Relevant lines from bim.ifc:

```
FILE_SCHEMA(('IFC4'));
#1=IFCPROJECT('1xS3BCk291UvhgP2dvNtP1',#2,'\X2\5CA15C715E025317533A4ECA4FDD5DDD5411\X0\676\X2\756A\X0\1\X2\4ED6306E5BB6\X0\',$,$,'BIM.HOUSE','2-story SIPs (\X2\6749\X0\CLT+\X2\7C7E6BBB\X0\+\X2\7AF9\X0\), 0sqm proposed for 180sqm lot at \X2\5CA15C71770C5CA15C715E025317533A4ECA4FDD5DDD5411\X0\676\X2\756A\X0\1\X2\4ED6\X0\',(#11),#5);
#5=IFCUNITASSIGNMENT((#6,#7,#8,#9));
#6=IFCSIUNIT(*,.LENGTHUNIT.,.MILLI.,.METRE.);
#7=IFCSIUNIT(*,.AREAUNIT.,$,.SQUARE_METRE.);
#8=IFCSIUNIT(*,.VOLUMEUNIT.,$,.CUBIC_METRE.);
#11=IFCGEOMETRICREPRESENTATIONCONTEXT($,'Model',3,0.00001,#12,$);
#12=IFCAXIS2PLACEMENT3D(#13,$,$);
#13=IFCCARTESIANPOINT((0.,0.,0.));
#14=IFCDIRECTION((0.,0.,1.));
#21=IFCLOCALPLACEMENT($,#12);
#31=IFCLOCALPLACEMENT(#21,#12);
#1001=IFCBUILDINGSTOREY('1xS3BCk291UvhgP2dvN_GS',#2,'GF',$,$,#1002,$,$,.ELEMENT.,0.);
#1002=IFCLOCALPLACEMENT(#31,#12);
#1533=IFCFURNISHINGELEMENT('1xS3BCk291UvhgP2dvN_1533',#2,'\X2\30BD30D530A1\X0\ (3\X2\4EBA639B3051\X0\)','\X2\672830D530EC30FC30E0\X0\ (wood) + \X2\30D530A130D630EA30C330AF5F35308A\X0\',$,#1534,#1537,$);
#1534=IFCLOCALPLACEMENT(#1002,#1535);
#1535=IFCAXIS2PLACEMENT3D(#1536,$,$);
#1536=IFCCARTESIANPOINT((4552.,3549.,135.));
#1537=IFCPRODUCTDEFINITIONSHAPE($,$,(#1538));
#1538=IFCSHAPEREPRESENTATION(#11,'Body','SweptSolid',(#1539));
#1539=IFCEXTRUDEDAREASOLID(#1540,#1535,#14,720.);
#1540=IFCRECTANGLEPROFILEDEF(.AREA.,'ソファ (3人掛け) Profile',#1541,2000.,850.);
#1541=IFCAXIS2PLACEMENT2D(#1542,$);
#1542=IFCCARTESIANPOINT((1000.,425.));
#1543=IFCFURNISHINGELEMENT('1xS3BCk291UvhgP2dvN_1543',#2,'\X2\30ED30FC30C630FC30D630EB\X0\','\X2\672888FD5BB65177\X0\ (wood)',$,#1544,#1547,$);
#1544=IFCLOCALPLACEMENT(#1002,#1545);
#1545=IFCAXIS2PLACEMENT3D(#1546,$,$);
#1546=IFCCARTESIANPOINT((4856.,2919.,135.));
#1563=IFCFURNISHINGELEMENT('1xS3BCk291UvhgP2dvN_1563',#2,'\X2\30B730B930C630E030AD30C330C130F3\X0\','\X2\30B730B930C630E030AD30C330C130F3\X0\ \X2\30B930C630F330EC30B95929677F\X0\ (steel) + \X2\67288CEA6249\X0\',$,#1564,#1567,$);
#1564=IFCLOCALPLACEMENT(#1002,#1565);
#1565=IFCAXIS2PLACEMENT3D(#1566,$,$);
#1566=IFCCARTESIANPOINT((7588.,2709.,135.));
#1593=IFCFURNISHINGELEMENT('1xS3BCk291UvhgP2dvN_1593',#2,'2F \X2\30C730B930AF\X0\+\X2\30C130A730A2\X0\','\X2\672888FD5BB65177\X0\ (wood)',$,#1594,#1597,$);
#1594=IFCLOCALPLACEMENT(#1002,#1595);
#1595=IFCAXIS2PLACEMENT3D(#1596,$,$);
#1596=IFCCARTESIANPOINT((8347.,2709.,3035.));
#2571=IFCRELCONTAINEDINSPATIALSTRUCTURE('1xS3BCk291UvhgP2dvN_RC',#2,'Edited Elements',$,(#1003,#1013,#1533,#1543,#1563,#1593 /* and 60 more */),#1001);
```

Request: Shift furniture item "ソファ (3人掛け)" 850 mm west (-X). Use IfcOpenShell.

```python
import ifcopenshell
import ifcopenshell.api.geometry
import ifcopenshell.util.placement

model = ifcopenshell.open("bim.ifc")

item = model.by_guid("1xS3BCk291UvhgP2dvN_1533")
matrix = ifcopenshell.util.placement.get_local_placement(item.ObjectPlacement)
matrix[0, 3] -= 850.0
ifcopenshell.api.geometry.edit_object_placement(model, product=item, matrix=matrix, is_si=False)

print(ifcopenshell.util.placement.get_local_placement(item.ObjectPlacement).round(3) + 0.0)

model.write("bim_edited.ifc")
```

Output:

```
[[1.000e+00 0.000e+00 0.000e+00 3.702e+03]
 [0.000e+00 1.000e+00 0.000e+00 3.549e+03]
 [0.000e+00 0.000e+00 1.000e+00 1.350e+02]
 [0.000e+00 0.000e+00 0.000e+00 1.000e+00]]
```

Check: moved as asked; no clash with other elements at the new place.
